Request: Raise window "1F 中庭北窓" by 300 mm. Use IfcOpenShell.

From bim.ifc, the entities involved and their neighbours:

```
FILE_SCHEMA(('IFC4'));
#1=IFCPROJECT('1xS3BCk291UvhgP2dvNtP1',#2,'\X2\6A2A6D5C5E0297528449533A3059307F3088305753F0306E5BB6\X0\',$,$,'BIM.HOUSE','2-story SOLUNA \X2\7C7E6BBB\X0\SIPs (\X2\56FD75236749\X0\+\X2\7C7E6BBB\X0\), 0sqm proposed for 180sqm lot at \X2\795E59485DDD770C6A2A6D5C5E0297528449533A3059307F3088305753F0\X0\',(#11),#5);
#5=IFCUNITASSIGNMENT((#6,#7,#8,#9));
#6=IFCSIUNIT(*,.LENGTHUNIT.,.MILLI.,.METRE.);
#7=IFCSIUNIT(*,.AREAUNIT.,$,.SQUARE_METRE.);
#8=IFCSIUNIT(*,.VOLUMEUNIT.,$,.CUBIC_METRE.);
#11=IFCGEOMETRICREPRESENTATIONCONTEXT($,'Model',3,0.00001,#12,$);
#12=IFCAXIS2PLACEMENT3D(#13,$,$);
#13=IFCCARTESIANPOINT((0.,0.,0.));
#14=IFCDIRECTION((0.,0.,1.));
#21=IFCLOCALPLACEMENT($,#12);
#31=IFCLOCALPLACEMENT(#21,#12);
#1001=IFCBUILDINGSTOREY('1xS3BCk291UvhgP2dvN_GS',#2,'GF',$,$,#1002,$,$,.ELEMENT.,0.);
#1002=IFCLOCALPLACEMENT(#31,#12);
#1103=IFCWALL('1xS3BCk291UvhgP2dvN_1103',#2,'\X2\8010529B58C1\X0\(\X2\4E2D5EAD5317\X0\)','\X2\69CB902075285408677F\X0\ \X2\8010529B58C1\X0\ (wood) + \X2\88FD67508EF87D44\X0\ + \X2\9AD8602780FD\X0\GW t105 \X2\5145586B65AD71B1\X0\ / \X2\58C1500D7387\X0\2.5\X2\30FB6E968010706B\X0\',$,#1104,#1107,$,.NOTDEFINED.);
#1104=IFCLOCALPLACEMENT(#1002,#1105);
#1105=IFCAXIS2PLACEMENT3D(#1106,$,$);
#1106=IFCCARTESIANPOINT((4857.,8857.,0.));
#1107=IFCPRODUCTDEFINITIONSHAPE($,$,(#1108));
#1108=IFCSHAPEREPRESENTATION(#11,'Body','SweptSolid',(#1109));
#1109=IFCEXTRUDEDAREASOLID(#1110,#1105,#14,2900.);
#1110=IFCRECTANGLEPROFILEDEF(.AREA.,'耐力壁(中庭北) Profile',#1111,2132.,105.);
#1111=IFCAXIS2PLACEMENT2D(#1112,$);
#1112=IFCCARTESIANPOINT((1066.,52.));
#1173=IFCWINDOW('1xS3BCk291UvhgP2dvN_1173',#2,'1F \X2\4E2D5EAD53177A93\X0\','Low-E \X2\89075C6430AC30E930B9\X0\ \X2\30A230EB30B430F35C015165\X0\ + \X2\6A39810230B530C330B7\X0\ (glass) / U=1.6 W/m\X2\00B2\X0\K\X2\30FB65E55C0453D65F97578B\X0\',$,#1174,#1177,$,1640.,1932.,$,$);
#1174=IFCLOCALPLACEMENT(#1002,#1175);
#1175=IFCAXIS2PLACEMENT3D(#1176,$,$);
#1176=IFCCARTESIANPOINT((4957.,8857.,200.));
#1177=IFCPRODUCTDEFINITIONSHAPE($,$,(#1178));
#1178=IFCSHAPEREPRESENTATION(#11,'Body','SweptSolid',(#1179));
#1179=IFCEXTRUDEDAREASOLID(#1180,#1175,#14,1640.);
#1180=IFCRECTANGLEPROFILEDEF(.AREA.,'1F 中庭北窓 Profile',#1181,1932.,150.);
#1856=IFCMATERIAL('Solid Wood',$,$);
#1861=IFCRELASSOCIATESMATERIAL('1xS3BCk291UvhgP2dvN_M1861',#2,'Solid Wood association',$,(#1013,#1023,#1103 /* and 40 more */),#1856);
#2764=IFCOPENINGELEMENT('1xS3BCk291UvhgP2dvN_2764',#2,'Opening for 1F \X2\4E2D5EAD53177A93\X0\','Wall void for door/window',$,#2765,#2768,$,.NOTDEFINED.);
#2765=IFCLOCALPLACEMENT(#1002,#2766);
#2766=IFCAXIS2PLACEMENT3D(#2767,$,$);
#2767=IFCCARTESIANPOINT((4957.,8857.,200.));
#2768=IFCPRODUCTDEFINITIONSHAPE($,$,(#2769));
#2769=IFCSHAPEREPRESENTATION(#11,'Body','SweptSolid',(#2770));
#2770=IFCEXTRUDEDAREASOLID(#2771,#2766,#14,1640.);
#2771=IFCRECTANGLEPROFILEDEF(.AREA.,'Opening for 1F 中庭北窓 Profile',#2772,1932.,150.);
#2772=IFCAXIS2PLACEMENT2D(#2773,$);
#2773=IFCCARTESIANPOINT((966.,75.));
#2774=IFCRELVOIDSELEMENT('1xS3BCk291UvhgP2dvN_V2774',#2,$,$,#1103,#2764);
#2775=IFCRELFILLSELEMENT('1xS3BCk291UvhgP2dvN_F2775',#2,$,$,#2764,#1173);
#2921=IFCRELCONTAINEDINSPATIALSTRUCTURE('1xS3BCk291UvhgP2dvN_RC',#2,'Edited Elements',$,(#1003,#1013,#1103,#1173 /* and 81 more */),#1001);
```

```python
import numpy as np
import ifcopenshell
import ifcopenshell.api.geometry
import ifcopenshell.util.placement
import ifcopenshell.util.unit

model = ifcopenshell.open("bim.ifc")
unit_scale = ifcopenshell.util.unit.calculate_unit_scale(model)

window = model.by_guid("1xS3BCk291UvhgP2dvN_1173")
opening = window.FillsVoids[0].RelatingOpeningElement
dz = 0.3 / unit_scale

shift = np.array([0.0, 0.0, dz])
# The window is not placed relative to its opening, so move both.
for product in (opening, window):
    matrix = ifcopenshell.util.placement.get_local_placement(product.ObjectPlacement)
    matrix[:3, 3] += shift
    ifcopenshell.api.geometry.edit_object_placement(model, product=product, matrix=matrix, is_si=False)

print(f"moved by {dz * unit_scale:+.3f} m")

model.write("bim-out.ifc")
```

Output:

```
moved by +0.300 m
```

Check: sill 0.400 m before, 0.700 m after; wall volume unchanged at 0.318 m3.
